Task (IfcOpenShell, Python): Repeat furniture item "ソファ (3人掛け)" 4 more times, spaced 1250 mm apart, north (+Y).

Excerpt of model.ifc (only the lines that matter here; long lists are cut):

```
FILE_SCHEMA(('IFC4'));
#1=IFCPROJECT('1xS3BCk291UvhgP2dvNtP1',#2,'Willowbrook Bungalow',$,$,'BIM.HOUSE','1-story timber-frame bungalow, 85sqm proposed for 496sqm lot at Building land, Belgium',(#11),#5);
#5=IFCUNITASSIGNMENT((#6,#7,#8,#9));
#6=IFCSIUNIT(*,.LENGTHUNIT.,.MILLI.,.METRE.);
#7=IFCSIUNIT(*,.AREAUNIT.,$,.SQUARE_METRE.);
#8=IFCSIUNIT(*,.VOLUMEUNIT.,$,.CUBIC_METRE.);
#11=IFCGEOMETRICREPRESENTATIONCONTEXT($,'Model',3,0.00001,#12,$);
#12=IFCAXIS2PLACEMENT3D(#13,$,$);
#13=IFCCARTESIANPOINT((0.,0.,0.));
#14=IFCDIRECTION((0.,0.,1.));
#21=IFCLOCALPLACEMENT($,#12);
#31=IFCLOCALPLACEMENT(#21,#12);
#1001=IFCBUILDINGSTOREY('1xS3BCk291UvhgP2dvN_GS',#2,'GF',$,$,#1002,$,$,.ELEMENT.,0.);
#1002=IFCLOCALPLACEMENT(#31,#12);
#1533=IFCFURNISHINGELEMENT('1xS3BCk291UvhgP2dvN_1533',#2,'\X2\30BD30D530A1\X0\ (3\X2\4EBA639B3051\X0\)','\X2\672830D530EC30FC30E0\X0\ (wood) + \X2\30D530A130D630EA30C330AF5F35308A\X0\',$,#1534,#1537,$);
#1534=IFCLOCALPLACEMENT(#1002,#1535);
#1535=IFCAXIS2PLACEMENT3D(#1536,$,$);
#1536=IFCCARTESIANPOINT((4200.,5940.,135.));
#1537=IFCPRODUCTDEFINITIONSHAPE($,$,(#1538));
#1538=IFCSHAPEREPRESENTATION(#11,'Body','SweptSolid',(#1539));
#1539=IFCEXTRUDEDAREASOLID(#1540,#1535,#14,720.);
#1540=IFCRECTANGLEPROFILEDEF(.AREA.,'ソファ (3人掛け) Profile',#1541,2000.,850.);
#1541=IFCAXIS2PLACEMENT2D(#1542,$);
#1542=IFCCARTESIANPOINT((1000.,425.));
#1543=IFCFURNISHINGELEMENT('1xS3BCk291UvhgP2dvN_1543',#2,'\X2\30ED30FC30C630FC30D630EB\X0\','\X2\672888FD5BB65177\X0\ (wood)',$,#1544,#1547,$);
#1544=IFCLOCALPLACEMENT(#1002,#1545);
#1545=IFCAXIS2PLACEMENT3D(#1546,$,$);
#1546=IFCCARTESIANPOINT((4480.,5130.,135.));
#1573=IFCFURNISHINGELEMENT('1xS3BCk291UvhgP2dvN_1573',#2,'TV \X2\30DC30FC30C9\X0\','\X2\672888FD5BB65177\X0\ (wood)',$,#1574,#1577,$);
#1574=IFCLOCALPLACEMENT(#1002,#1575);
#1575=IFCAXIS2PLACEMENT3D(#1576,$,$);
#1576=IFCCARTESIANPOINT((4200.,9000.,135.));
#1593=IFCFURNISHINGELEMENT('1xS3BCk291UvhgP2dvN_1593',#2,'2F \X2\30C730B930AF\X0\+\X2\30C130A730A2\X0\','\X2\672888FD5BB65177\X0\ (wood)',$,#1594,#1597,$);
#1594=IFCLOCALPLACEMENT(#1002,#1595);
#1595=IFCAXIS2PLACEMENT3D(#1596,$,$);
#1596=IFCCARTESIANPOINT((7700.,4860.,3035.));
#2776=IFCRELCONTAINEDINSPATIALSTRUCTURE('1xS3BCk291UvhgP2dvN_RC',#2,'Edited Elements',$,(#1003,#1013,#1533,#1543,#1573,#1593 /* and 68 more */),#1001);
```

```python
import numpy as np
import ifcopenshell
import ifcopenshell.api.geometry
import ifcopenshell.api.root
import ifcopenshell.util.element
import ifcopenshell.util.placement

model = ifcopenshell.open("model.ifc")


def reuse_history(source, copy):
    """copy_class also copies each property set's owner history, people and application; keep the originals."""
    for rel in copy.IsDefinedBy:
        if rel.is_a("IfcRelDefinesByProperties") and (history := rel.RelatingPropertyDefinition.OwnerHistory):
            rel.RelatingPropertyDefinition.OwnerHistory = source.OwnerHistory
            ifcopenshell.util.element.remove_deep2(model, history)


source = model.by_guid("1xS3BCk291UvhgP2dvN_1533")
base = ifcopenshell.util.placement.get_local_placement(source.ObjectPlacement)
step = np.array([0.0, 1.0, 0.0]) * 1250.0

for i in range(1, 5):
    copy = ifcopenshell.api.root.copy_class(model, product=source)
    copy.Representation = ifcopenshell.util.element.copy_deep(
        model, source.Representation, exclude=["IfcGeometricRepresentationContext", "IfcRepresentationMap"]
    )
    reuse_history(source, copy)
    matrix = base.copy()
    matrix[:3, 3] += i * step
    print("added at", matrix[:3, 3].round(3) + 0.0)
    ifcopenshell.api.geometry.edit_object_placement(model, product=copy, matrix=matrix, is_si=False)

model.write("model_rev.ifc")
```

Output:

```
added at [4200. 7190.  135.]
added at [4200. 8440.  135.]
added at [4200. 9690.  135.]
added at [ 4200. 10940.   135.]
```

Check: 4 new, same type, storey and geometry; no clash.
